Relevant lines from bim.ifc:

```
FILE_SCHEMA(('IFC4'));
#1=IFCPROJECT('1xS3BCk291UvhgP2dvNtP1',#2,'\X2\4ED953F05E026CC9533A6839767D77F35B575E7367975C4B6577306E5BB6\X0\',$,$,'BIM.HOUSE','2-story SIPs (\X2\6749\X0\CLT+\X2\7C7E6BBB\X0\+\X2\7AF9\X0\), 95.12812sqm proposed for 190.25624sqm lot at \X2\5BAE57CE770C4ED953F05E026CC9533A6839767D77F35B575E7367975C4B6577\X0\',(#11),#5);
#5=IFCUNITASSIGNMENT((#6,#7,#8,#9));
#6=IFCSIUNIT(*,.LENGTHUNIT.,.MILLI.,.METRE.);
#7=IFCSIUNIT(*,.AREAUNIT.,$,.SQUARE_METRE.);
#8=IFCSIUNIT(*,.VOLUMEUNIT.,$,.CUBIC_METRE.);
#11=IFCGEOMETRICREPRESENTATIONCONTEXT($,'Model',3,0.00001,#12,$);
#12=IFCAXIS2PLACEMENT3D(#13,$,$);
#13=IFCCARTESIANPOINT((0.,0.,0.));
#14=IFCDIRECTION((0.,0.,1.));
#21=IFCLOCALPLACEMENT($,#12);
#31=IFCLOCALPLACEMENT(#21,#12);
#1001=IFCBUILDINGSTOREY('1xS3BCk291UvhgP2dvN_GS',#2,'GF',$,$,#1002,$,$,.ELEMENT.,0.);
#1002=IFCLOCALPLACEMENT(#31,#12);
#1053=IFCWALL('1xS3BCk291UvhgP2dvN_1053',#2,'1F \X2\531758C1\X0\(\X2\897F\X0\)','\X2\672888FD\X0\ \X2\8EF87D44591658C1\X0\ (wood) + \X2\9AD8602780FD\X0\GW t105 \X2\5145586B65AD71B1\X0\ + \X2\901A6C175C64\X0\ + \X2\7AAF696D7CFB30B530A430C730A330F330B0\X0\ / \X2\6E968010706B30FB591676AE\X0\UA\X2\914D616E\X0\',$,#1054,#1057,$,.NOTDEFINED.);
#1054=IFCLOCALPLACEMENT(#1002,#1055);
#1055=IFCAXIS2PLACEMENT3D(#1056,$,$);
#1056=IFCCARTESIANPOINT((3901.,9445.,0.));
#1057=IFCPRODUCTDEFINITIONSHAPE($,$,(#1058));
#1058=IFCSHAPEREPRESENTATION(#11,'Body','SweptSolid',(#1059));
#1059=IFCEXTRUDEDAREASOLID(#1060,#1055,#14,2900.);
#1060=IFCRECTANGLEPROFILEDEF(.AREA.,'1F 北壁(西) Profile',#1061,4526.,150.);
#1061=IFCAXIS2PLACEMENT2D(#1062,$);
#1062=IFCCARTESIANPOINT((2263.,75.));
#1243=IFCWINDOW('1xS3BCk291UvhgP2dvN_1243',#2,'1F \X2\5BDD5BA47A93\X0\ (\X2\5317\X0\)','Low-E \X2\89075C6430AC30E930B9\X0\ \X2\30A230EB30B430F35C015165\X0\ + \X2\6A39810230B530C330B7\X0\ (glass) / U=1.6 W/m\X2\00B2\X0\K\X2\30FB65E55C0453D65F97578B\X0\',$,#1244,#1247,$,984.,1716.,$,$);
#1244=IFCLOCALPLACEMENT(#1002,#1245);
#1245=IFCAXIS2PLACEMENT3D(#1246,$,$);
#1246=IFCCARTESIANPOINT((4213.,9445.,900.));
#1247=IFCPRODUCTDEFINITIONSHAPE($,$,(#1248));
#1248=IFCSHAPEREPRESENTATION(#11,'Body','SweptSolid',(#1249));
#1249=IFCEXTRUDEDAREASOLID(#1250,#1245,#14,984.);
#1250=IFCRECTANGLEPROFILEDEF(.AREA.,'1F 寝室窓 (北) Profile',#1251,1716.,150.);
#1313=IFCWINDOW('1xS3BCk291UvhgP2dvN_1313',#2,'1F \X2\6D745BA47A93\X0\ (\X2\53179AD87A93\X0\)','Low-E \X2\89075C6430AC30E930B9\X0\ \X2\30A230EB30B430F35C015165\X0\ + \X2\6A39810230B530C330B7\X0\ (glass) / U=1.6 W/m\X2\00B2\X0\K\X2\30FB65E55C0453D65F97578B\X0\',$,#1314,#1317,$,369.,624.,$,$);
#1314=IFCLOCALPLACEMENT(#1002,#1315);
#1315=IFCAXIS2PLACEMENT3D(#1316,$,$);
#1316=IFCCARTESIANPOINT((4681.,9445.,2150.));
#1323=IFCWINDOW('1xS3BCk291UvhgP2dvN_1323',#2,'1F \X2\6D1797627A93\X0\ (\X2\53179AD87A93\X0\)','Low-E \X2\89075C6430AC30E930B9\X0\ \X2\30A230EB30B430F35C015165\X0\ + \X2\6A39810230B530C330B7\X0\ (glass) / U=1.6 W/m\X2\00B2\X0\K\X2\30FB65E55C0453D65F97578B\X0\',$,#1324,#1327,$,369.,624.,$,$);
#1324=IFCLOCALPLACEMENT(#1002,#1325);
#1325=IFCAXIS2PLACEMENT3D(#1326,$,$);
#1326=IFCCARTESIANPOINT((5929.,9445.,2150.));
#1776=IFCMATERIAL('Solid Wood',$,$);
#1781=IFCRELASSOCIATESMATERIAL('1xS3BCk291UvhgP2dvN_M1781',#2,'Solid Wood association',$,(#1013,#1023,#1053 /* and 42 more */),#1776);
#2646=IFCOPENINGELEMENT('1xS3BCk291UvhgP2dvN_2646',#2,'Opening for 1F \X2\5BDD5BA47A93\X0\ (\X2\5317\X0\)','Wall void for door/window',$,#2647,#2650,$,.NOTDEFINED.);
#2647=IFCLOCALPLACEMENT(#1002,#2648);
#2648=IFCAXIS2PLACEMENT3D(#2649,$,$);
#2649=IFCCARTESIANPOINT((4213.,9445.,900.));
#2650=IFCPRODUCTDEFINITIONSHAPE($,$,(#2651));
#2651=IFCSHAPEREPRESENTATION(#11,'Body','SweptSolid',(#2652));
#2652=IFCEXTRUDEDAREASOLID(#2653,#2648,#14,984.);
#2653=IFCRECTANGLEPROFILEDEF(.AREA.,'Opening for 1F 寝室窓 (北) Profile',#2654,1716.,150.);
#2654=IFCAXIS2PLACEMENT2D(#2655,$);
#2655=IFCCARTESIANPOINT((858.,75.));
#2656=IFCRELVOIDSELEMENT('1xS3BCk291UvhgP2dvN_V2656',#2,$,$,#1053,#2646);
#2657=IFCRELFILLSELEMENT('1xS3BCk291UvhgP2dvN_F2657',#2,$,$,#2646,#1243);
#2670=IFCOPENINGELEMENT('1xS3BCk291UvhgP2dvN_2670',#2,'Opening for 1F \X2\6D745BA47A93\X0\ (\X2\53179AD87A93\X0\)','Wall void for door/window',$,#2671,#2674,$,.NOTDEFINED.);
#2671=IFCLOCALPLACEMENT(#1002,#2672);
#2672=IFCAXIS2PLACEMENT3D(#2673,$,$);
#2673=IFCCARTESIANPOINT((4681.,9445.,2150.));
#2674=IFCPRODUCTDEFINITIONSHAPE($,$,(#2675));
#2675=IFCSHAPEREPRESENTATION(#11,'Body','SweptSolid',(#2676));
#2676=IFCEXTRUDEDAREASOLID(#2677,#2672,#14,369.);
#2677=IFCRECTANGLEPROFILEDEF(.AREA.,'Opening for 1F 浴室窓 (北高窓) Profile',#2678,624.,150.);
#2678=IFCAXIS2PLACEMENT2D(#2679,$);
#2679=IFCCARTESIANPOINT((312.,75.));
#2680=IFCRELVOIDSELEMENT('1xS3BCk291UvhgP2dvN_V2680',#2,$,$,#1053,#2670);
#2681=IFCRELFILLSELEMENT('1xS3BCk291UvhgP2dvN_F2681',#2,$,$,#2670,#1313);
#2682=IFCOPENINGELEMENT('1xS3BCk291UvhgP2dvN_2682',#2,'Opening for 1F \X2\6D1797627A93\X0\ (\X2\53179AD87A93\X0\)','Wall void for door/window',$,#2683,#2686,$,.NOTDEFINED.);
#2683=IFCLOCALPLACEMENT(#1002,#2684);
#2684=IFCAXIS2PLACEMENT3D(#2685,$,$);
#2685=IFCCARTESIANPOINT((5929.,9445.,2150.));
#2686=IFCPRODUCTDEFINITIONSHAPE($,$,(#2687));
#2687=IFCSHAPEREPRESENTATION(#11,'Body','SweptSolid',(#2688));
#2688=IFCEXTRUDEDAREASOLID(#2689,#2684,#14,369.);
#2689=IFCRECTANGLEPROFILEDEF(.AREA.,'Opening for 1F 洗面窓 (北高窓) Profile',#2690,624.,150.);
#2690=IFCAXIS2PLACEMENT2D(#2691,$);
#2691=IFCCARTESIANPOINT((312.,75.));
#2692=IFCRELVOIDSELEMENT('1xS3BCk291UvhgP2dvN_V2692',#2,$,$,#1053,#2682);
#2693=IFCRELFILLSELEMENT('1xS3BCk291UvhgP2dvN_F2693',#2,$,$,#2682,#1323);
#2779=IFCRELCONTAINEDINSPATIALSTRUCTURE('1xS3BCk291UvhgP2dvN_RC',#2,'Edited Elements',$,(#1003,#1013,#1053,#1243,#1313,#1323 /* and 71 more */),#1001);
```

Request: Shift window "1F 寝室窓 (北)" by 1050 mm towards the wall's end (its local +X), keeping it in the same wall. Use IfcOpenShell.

```python
import ifcopenshell
import ifcopenshell.api.geometry
import ifcopenshell.util.placement
import ifcopenshell.util.unit

model = ifcopenshell.open("bim.ifc")
unit_scale = ifcopenshell.util.unit.calculate_unit_scale(model)

window = model.by_id(1243)
opening = window.FillsVoids[0].RelatingOpeningElement
wall = opening.VoidsElements[0].RelatingBuildingElement

wall_matrix = ifcopenshell.util.placement.get_local_placement(wall.ObjectPlacement)
shift = wall_matrix[:3, 0] * 1.05 / unit_scale
before = ifcopenshell.util.placement.get_local_placement(window.ObjectPlacement)[:3, 3].copy()

# The window is not placed relative to its opening, so move both.
for product in (opening, window):
    matrix = ifcopenshell.util.placement.get_local_placement(product.ObjectPlacement)
    matrix[:3, 3] += shift
    ifcopenshell.api.geometry.edit_object_placement(model, product=product, matrix=matrix, is_si=False)

after = ifcopenshell.util.placement.get_local_placement(window.ObjectPlacement)[:3, 3]
print("window moved by", (after - before).round(3) + 0.0)

model.write("bim_rev.ifc")
```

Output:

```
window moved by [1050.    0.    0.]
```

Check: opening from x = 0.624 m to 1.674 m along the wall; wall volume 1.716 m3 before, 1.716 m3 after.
